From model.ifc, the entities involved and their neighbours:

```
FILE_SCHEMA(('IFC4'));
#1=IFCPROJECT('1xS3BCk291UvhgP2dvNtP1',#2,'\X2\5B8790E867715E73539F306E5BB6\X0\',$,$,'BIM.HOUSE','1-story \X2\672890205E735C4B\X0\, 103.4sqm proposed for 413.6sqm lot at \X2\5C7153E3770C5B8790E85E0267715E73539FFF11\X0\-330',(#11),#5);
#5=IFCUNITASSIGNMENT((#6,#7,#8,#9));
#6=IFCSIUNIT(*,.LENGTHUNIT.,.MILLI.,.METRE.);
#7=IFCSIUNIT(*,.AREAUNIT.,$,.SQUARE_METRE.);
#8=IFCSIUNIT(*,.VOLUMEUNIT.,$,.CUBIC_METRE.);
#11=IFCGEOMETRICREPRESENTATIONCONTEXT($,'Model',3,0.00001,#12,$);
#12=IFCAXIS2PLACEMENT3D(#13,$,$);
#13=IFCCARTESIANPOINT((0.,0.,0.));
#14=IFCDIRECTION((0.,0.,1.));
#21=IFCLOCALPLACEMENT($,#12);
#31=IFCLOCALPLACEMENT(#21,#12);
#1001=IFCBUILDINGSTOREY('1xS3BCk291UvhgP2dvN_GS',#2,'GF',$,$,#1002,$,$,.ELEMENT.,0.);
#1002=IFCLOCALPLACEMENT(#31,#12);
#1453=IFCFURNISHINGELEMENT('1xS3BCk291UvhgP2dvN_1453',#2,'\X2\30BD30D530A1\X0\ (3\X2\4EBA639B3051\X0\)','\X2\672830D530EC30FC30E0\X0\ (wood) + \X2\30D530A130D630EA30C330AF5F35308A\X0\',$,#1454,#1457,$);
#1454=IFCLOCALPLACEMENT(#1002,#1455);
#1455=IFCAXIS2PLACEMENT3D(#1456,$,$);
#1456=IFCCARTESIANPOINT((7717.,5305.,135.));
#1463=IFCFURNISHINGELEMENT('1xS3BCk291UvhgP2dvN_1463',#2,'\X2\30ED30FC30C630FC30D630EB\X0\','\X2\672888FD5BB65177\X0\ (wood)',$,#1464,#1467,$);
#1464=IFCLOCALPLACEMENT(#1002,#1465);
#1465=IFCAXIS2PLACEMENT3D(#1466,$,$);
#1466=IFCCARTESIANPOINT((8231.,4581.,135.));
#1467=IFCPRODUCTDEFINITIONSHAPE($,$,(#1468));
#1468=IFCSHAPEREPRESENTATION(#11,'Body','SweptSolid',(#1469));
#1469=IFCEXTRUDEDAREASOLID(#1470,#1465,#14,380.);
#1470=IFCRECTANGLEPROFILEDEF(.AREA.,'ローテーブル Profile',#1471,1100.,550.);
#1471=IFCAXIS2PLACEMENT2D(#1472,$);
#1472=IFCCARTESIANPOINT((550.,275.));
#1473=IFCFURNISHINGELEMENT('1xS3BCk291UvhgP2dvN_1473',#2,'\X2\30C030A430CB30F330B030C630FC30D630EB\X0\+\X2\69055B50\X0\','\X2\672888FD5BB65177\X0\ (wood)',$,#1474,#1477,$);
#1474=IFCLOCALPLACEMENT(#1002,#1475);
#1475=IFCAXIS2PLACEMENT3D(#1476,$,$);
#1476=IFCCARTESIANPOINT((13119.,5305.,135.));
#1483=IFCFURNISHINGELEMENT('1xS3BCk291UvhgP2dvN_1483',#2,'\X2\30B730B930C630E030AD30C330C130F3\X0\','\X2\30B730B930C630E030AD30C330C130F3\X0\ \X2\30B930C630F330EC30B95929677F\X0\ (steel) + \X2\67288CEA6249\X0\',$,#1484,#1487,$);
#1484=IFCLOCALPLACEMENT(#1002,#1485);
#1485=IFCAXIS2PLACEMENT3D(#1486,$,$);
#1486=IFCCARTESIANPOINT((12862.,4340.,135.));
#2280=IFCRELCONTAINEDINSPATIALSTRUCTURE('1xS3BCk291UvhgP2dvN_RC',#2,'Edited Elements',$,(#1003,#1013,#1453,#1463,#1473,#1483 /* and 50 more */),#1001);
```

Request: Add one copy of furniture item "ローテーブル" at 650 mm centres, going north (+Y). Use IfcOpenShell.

```python
import numpy as np
import ifcopenshell
import ifcopenshell.api.geometry
import ifcopenshell.api.root
import ifcopenshell.util.element
import ifcopenshell.util.placement
import ifcopenshell.util.unit

model = ifcopenshell.open("model.ifc")
unit_scale = ifcopenshell.util.unit.calculate_unit_scale(model)


def reuse_history(source, copy):
    """copy_class also copies each property set's owner history, people and application; keep the originals."""
    for rel in copy.IsDefinedBy:
        if rel.is_a("IfcRelDefinesByProperties") and (history := rel.RelatingPropertyDefinition.OwnerHistory):
            rel.RelatingPropertyDefinition.OwnerHistory = source.OwnerHistory
            ifcopenshell.util.element.remove_deep2(model, history)


source = model.by_guid("1xS3BCk291UvhgP2dvN_1463")
base = ifcopenshell.util.placement.get_local_placement(source.ObjectPlacement)
step = np.array([0.0, 1.0, 0.0]) * 0.65 / unit_scale

for i in range(1, 2):
    copy = ifcopenshell.api.root.copy_class(model, product=source)
    copy.Representation = ifcopenshell.util.element.copy_deep(
        model, source.Representation, exclude=["IfcGeometricRepresentationContext", "IfcRepresentationMap"]
    )
    reuse_history(source, copy)
    matrix = base.copy()
    matrix[:3, 3] += i * step
    print("added at", matrix[:3, 3].round(3) + 0.0)
    ifcopenshell.api.geometry.edit_object_placement(model, product=copy, matrix=matrix, is_si=False)

model.write("model-out.ifc")
```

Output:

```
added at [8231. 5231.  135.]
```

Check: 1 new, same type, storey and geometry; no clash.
